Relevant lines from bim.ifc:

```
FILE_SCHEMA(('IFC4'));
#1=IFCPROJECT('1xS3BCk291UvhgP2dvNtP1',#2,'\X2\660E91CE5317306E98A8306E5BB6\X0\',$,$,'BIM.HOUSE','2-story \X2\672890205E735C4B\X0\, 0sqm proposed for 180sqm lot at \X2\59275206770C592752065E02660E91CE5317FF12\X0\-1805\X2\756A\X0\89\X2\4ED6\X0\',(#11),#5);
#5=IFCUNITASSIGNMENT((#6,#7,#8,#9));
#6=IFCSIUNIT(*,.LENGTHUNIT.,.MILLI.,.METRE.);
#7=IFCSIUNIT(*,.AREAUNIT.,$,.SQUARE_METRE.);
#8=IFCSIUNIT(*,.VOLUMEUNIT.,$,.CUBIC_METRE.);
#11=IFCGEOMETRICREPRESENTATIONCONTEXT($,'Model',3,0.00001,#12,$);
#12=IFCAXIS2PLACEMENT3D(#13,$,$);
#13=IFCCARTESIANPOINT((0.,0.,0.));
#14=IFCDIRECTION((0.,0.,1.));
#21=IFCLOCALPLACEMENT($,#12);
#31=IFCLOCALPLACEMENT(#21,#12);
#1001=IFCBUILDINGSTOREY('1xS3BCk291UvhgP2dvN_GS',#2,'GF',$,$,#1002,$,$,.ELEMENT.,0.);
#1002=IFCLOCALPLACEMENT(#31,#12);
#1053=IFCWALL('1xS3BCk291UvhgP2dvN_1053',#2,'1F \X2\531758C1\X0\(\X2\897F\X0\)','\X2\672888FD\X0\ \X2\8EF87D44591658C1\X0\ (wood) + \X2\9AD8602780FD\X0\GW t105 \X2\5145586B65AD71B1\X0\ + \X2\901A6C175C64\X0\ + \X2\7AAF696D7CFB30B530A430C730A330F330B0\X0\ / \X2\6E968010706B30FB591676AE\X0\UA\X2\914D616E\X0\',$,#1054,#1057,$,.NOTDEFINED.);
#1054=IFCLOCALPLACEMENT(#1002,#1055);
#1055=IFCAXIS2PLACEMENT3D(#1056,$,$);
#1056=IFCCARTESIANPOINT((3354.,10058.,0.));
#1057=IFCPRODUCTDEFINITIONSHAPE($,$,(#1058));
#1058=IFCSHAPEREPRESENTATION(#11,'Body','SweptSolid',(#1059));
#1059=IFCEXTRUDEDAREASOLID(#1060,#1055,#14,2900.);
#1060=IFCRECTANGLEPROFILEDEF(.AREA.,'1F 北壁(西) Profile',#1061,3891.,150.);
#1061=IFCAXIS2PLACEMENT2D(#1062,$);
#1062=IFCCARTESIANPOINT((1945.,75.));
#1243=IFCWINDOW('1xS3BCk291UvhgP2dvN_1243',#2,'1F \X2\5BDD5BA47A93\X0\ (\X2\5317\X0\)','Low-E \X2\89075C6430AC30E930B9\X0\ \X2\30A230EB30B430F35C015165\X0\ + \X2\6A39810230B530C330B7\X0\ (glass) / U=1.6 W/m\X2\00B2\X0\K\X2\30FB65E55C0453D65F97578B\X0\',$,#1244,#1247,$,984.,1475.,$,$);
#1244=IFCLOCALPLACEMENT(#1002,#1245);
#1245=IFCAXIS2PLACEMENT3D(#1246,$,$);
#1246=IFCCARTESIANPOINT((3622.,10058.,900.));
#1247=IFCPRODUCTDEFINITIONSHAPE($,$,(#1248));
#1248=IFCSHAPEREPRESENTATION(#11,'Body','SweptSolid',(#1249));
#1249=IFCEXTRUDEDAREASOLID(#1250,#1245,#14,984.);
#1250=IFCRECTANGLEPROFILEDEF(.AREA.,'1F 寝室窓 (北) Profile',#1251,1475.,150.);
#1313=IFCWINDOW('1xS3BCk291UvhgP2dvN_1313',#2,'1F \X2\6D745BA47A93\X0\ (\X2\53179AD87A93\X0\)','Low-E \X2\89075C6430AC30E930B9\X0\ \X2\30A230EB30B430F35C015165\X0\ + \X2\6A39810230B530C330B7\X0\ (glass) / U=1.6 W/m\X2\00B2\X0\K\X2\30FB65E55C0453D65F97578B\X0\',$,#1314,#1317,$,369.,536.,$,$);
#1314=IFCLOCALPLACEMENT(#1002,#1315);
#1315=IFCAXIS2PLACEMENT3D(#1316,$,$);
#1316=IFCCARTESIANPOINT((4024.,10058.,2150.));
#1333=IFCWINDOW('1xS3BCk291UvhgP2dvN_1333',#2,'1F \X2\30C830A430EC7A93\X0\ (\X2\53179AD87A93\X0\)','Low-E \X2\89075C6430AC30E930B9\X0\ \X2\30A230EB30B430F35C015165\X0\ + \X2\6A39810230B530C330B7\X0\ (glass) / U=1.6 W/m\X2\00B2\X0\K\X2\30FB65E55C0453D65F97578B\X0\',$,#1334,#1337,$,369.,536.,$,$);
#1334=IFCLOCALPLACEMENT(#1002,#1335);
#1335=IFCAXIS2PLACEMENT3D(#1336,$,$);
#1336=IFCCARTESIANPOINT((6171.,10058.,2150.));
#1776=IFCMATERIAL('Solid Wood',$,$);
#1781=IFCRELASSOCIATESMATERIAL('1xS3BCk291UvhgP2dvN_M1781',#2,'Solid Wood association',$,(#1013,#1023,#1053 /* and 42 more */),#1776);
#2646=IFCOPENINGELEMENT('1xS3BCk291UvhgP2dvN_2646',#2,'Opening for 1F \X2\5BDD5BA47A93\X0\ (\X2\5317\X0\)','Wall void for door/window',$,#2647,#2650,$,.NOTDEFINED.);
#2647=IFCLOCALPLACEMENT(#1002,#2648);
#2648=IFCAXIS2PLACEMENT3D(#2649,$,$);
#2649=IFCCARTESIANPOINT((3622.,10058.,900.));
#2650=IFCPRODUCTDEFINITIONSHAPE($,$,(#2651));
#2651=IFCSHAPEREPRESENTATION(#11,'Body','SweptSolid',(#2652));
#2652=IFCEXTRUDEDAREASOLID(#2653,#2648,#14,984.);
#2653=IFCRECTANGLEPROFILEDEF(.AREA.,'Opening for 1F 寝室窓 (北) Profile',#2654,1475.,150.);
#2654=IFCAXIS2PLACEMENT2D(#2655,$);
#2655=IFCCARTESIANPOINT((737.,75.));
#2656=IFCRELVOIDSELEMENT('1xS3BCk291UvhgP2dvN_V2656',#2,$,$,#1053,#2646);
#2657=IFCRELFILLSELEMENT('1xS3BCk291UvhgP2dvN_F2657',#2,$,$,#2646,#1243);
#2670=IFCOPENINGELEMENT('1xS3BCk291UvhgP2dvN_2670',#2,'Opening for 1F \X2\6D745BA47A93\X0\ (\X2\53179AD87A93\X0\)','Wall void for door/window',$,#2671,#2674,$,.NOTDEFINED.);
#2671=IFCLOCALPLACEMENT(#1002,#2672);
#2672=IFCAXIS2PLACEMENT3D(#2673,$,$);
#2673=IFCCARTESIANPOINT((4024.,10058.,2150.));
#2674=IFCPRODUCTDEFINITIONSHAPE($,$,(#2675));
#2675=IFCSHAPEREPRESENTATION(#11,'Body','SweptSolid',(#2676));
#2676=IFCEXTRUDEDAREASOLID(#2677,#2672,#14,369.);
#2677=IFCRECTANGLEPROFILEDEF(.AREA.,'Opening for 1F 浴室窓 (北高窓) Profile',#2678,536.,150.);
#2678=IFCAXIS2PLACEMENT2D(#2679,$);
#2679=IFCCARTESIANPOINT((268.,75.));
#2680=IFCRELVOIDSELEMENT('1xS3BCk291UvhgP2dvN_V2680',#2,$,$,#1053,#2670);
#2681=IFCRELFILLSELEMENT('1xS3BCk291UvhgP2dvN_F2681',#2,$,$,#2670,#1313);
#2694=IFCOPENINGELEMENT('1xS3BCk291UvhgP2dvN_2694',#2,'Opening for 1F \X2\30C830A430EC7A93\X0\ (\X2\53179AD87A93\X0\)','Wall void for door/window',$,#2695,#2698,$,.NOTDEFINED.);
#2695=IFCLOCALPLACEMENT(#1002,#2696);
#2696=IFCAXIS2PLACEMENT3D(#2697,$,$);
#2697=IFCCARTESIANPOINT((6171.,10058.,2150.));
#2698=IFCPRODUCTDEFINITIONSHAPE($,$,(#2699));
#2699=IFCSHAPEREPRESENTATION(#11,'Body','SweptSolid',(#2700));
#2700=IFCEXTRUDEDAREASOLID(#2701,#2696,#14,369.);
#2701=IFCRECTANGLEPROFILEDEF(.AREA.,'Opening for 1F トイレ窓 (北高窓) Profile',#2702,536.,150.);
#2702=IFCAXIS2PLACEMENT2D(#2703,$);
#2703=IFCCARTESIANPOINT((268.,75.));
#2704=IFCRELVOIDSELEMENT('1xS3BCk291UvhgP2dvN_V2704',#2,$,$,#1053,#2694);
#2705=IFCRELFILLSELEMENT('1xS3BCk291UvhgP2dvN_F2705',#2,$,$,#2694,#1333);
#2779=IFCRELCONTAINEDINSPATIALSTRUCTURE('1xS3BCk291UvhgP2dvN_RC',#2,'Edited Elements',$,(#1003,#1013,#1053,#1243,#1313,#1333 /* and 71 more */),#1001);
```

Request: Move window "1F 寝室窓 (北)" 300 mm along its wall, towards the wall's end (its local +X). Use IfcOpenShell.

```python
import ifcopenshell
import ifcopenshell.api.geometry
import ifcopenshell.util.placement
import ifcopenshell.util.unit

model = ifcopenshell.open("bim.ifc")
unit_scale = ifcopenshell.util.unit.calculate_unit_scale(model)

window = model.by_guid("1xS3BCk291UvhgP2dvN_1243")
opening = window.FillsVoids[0].RelatingOpeningElement
wall = opening.VoidsElements[0].RelatingBuildingElement

wall_matrix = ifcopenshell.util.placement.get_local_placement(wall.ObjectPlacement)
shift = wall_matrix[:3, 0] * 0.3 / unit_scale
before = ifcopenshell.util.placement.get_local_placement(window.ObjectPlacement)[:3, 3].copy()

# The window is not placed relative to its opening, so move both.
for product in (opening, window):
    matrix = ifcopenshell.util.placement.get_local_placement(product.ObjectPlacement)
    matrix[:3, 3] += shift
    ifcopenshell.api.geometry.edit_object_placement(model, product=product, matrix=matrix, is_si=False)

after = ifcopenshell.util.placement.get_local_placement(window.ObjectPlacement)[:3, 3]
print("window moved by", (after - before).round(3) + 0.0)

model.write("bim_rev.ifc")
```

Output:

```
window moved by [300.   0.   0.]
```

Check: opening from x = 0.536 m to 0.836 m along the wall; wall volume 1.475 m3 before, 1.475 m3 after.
